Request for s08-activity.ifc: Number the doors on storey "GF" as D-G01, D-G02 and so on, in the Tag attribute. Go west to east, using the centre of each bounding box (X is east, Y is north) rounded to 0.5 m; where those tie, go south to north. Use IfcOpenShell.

First a look at what the model holds.

```python
import ifcopenshell
import ifcopenshell.util.element
import ifcopenshell.util.placement

model = ifcopenshell.open("s08-activity.ifc")
print(model.schema)
storey = next(s for s in model.by_type("IfcBuildingStorey") if s.Name == "GF")
doors = [e for e in ifcopenshell.util.element.get_decomposition(storey) if e.is_a("IfcDoor")]
for e in sorted(doors, key=lambda e: e.id()):
    origin = ifcopenshell.util.placement.get_local_placement(e.ObjectPlacement)[:3, 3]
    print(e.id(), e.Tag, e.Name, origin.round(2) + 0.0, sep=" | ")
```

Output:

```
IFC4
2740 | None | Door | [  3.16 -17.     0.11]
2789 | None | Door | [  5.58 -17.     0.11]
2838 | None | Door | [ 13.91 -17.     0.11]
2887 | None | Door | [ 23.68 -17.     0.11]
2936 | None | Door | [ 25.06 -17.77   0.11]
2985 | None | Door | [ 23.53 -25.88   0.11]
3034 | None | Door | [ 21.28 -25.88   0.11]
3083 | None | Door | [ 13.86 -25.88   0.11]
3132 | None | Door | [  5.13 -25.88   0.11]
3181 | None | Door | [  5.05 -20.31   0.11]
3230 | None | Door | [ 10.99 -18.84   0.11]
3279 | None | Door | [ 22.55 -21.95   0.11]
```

```python
import ifcopenshell
import ifcopenshell.geom
import ifcopenshell.util.element
import ifcopenshell.util.shape

model = ifcopenshell.open("s08-activity.ifc")
settings = ifcopenshell.geom.settings()
settings.set("use-world-coords", True)


def centre(element):
    shape = ifcopenshell.geom.create_shape(settings, element)
    return ifcopenshell.util.shape.get_bbox_centroid(shape.geometry)


storey = next(s for s in model.by_type("IfcBuildingStorey") if s.Name == "GF")
doors = [e for e in ifcopenshell.util.element.get_decomposition(storey) if e.is_a("IfcDoor")]

# Insertion points can sit at a corner or the storey origin, so sort by the geometry (in metres).
centres = {e: centre(e) for e in doors}
doors.sort(key=lambda e: (round(centres[e][0] / 0.5), centres[e][1]))

for i, e in enumerate(doors, start=1):
    number = f"D-G{i:02d}"
    e.Tag = number
    print(e.id(), number)

model.write("s08-activity_updated.ifc")
```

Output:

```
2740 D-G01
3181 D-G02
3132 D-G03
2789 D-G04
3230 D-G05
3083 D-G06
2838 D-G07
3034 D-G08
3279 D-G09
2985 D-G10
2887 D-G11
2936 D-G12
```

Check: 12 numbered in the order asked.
